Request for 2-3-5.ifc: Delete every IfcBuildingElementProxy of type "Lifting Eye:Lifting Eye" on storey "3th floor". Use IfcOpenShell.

First a look at what the model holds.

```python
import ifcopenshell
import ifcopenshell.util.element

model = ifcopenshell.open("2-3-5.ifc")
print(model.schema)
storey = next(s for s in model.by_type("IfcBuildingStorey") if s.Name == "3th floor")
proxies = [e for e in ifcopenshell.util.element.get_decomposition(storey) if e.is_a("IfcBuildingElementProxy")]
seen = {}
for e in proxies:
    element_type = ifcopenshell.util.element.get_type(e)
    name = element_type.Name if element_type not in (None, e) else None
    seen[name] = seen.get(name, 0) + 1
for name, count in sorted(seen.items(), key=str):
    print(count, "x", name)
```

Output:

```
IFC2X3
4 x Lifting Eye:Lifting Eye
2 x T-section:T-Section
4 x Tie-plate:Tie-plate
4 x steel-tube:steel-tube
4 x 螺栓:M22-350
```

```python
import ifcopenshell
import ifcopenshell.api.root
import ifcopenshell.util.element

model = ifcopenshell.open("2-3-5.ifc")

storey = next(s for s in model.by_type("IfcBuildingStorey") if s.Name == "3th floor")
proxies = [e for e in ifcopenshell.util.element.get_decomposition(storey) if e.is_a("IfcBuildingElementProxy")]
targets = [e for e in proxies if (t := ifcopenshell.util.element.get_type(e)) not in (None, e) and t.Name == "Lifting Eye:Lifting Eye"]

for e in targets:
    ifcopenshell.api.root.remove_product(model, product=e)
print(len(targets), "removed")

model.write("2-3-5-out.ifc")
```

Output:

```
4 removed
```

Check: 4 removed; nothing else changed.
